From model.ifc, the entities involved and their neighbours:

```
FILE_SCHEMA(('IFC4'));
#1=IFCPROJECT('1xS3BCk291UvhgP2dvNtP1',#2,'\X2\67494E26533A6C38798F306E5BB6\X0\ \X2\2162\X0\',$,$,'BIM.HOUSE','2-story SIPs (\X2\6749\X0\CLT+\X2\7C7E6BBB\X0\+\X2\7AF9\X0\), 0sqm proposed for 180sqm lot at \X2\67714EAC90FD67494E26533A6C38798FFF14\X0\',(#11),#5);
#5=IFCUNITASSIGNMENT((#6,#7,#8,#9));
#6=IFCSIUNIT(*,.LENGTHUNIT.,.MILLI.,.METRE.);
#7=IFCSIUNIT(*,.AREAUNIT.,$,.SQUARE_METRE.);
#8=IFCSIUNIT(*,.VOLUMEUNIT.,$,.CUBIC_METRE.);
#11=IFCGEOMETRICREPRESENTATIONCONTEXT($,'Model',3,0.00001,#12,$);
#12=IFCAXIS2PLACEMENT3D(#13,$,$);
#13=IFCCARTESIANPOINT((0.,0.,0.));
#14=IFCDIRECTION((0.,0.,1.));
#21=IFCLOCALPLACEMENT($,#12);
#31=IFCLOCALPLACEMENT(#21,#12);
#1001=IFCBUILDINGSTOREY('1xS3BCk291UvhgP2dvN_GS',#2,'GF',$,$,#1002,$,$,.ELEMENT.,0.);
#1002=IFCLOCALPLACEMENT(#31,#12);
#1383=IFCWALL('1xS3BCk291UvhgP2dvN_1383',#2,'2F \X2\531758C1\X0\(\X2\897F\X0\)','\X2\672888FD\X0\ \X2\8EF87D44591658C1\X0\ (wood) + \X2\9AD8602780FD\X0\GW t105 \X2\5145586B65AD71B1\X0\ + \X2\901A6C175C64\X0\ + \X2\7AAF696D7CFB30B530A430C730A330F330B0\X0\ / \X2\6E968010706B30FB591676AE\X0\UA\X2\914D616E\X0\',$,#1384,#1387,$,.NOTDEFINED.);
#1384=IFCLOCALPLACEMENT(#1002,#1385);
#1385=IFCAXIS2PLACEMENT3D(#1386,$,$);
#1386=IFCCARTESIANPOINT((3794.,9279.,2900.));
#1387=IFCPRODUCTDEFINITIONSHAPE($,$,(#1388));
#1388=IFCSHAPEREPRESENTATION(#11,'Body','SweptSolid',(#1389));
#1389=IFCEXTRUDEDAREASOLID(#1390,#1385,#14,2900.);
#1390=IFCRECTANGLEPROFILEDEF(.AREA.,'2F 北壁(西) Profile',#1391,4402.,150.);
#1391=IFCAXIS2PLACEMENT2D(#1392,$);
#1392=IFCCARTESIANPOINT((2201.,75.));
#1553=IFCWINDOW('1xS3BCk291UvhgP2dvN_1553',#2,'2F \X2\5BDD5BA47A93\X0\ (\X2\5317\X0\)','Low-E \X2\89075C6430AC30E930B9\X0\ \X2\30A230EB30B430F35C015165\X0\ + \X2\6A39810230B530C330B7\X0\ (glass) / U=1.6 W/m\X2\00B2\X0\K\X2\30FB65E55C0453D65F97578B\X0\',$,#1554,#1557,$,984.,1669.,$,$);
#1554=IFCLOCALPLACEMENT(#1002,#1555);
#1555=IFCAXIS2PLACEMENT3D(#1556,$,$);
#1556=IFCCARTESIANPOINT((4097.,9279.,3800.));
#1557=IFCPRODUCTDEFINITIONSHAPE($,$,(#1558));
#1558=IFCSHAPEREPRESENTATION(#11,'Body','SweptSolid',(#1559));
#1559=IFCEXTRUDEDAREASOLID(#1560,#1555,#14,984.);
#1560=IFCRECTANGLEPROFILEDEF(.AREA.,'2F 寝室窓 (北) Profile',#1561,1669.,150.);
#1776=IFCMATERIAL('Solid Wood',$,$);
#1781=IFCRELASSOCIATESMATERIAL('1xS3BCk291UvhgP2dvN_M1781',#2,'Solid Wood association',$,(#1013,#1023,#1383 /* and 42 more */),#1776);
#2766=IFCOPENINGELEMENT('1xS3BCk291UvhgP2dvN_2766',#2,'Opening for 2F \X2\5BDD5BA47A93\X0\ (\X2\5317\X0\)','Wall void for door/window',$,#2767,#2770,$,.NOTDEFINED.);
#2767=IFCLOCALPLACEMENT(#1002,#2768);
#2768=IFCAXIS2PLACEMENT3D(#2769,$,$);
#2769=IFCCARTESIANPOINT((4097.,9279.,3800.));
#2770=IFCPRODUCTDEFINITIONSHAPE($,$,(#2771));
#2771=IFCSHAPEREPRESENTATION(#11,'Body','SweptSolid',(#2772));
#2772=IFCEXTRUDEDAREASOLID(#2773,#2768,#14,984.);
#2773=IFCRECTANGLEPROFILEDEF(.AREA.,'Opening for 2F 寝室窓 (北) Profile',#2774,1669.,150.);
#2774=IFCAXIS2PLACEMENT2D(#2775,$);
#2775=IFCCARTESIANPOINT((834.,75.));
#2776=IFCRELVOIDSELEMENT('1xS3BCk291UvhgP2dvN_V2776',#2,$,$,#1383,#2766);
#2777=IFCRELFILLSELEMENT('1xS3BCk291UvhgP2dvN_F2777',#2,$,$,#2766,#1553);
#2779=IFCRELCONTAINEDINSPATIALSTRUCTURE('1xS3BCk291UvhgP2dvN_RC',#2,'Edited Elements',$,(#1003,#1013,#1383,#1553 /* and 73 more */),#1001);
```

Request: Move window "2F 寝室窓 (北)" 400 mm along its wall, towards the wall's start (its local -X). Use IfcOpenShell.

```python
import ifcopenshell
import ifcopenshell.api.geometry
import ifcopenshell.util.placement
import ifcopenshell.util.unit

model = ifcopenshell.open("model.ifc")
unit_scale = ifcopenshell.util.unit.calculate_unit_scale(model)

window = model.by_guid("1xS3BCk291UvhgP2dvN_1553")
opening = window.FillsVoids[0].RelatingOpeningElement
wall = opening.VoidsElements[0].RelatingBuildingElement

wall_matrix = ifcopenshell.util.placement.get_local_placement(wall.ObjectPlacement)
shift = wall_matrix[:3, 0] * -0.4 / unit_scale
before = ifcopenshell.util.placement.get_local_placement(window.ObjectPlacement)[:3, 3].copy()

# The window is not placed relative to its opening, so move both.
for product in (opening, window):
    matrix = ifcopenshell.util.placement.get_local_placement(product.ObjectPlacement)
    matrix[:3, 3] += shift
    ifcopenshell.api.geometry.edit_object_placement(model, product=product, matrix=matrix, is_si=False)

after = ifcopenshell.util.placement.get_local_placement(window.ObjectPlacement)[:3, 3]
print("window moved by", (after - before).round(3) + 0.0)

model.write("model-out.ifc")
```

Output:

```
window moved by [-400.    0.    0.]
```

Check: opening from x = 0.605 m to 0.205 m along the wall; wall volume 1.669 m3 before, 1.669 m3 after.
